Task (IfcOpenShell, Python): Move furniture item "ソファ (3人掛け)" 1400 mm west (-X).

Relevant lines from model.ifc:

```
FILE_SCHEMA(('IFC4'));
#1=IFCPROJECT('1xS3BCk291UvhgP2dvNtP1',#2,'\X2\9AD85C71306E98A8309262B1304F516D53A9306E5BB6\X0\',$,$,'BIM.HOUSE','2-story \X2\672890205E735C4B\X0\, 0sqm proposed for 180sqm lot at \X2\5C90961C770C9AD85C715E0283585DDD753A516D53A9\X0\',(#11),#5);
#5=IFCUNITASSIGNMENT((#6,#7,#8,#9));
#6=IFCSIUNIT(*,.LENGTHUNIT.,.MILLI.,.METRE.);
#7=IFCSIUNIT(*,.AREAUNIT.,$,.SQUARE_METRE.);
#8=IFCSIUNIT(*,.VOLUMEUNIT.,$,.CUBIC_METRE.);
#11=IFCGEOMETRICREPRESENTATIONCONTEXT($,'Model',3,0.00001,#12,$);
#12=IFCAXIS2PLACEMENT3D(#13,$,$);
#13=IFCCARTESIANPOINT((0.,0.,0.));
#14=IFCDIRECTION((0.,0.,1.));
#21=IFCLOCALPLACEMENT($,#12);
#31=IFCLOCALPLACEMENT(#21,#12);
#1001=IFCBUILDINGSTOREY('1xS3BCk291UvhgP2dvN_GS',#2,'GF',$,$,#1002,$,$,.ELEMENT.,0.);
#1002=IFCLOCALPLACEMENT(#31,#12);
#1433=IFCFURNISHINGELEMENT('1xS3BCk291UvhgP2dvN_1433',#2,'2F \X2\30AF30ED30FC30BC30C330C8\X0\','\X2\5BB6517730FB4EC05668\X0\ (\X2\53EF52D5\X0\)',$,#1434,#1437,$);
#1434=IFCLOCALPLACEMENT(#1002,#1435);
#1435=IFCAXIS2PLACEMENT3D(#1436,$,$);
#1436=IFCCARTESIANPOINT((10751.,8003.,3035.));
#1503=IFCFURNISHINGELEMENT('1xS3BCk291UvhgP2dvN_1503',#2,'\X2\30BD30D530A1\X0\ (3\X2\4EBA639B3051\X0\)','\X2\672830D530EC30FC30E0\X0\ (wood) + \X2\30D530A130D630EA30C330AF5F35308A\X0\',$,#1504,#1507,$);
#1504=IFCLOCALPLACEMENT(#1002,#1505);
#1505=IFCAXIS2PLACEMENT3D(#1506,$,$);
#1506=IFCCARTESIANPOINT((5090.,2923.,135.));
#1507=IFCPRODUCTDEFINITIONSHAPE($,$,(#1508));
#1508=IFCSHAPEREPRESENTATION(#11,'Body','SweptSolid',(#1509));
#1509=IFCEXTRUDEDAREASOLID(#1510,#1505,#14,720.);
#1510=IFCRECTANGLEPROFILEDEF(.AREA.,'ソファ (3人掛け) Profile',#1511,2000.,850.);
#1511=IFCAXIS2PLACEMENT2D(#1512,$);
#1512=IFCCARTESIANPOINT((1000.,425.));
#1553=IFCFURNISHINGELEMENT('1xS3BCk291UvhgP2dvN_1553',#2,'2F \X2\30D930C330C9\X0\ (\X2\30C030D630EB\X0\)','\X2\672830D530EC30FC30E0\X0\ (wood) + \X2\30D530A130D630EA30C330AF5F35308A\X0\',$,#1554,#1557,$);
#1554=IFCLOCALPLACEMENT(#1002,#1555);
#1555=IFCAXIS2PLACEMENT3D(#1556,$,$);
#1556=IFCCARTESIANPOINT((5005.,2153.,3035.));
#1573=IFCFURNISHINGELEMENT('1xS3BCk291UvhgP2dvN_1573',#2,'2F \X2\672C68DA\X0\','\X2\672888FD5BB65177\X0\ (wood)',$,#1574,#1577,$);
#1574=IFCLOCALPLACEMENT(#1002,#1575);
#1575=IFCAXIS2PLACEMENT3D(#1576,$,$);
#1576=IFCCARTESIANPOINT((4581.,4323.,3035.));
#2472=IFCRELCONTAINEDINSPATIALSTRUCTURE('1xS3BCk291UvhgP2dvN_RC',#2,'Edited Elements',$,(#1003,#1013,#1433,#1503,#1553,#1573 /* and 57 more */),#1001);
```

```python
import ifcopenshell
import ifcopenshell.api.geometry
import ifcopenshell.util.placement
import ifcopenshell.util.unit

model = ifcopenshell.open("model.ifc")
unit_scale = ifcopenshell.util.unit.calculate_unit_scale(model)

item = model.by_guid("1xS3BCk291UvhgP2dvN_1503")
matrix = ifcopenshell.util.placement.get_local_placement(item.ObjectPlacement)
matrix[0, 3] -= 1.4 / unit_scale
ifcopenshell.api.geometry.edit_object_placement(model, product=item, matrix=matrix, is_si=False)

print(ifcopenshell.util.placement.get_local_placement(item.ObjectPlacement).round(3) + 0.0)

model.write("model_edited.ifc")
```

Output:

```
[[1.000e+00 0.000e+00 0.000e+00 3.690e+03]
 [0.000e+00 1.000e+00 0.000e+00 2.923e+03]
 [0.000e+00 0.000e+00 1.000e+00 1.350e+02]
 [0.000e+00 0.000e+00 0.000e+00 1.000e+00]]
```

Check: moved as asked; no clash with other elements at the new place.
